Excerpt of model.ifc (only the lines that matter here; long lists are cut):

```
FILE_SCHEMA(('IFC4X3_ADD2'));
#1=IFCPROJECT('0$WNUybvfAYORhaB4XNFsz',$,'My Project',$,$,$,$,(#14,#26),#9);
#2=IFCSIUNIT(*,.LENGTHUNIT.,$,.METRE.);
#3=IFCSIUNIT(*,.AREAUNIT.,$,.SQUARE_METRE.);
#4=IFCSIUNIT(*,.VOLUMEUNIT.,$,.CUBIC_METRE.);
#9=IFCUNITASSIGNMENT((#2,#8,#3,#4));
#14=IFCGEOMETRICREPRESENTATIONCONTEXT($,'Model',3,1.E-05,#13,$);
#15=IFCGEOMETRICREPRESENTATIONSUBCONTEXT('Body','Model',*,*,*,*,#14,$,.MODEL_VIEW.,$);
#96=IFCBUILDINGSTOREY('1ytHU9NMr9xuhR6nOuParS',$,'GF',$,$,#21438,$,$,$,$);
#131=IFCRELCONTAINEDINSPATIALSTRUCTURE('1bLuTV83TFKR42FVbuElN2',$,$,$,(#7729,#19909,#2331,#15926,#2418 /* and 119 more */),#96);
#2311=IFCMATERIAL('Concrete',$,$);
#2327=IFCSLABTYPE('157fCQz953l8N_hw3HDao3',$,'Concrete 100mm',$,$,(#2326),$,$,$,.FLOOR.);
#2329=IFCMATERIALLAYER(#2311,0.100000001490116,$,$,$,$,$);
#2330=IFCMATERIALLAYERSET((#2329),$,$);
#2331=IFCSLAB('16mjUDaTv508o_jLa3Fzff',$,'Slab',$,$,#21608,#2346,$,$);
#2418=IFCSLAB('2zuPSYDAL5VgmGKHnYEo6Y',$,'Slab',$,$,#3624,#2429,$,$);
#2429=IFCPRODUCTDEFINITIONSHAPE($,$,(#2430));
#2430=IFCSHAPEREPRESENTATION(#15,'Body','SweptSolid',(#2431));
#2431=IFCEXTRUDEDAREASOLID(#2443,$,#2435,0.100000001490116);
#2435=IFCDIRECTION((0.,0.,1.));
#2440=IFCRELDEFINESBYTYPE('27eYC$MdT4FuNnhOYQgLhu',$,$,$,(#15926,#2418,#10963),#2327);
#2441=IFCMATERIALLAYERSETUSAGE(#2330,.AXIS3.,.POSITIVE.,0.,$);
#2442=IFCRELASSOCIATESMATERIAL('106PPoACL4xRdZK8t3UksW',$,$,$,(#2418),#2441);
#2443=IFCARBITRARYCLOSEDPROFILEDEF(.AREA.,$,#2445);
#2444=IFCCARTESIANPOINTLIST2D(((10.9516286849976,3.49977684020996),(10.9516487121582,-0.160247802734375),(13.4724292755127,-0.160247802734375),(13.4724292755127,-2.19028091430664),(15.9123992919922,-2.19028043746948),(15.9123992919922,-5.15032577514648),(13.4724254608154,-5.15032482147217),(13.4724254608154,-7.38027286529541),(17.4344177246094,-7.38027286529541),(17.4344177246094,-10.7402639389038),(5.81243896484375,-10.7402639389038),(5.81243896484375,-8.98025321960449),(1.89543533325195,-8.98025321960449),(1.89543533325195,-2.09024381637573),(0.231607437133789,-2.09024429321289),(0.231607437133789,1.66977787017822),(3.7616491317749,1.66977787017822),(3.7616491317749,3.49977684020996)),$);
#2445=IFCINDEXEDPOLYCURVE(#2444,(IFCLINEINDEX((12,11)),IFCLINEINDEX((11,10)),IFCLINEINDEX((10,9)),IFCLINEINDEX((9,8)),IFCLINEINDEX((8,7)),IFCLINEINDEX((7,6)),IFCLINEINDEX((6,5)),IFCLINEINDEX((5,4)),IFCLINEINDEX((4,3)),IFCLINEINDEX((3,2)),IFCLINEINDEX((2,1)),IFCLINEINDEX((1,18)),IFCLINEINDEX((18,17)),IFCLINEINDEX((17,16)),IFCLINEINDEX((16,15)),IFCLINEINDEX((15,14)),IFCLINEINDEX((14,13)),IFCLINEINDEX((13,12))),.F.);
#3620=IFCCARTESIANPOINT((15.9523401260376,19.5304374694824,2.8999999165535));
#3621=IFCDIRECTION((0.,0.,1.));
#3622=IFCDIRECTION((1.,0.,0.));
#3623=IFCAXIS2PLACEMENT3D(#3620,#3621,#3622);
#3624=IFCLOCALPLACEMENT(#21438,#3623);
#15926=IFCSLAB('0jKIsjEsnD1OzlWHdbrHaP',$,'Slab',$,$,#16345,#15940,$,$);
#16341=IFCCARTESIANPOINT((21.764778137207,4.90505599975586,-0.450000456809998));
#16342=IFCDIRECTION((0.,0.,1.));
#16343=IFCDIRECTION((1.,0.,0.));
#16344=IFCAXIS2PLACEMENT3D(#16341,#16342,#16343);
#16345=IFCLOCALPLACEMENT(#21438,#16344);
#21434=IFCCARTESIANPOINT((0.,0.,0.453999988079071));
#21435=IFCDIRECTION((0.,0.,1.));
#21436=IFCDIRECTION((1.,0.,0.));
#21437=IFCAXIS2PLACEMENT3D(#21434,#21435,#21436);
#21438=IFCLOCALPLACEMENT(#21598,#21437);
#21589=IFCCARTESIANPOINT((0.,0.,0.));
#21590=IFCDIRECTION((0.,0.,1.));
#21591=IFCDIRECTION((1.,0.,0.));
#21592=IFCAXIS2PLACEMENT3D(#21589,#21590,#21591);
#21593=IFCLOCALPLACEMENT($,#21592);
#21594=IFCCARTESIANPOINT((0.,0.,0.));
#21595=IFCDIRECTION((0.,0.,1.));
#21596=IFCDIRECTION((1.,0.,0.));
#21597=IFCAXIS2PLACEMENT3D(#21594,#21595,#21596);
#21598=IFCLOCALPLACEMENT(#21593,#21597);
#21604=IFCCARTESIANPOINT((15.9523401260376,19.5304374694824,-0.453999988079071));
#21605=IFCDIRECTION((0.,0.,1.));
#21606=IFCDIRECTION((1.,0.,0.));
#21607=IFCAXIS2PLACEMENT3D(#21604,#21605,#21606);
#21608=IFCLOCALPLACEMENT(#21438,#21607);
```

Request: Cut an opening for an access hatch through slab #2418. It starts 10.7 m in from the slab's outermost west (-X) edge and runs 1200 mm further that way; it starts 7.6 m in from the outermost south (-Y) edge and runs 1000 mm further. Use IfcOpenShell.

```python
import numpy as np
import ifcopenshell
import ifcopenshell.api.feature
import ifcopenshell.api.geometry
import ifcopenshell.api.root
import ifcopenshell.geom
import ifcopenshell.util.placement
import ifcopenshell.util.representation
import ifcopenshell.util.shape
import ifcopenshell.util.unit

model = ifcopenshell.open("model.ifc")
unit_scale = ifcopenshell.util.unit.calculate_unit_scale(model)
settings = ifcopenshell.geom.settings()


def volume(element):
    """Net volume in cubic metres, openings subtracted."""
    shape = ifcopenshell.geom.create_shape(settings, element)
    return ifcopenshell.util.shape.get_volume(shape.geometry)


slab = model.by_guid("2zuPSYDAL5VgmGKHnYEo6Y")
before = volume(slab)

# Extent in the slab's own axes, in metres. The edges named are its -X and -Y sides.
slab_shape = ifcopenshell.geom.create_shape(settings, slab)
vertices = ifcopenshell.util.shape.get_vertices(slab_shape.geometry)
x_min, y_min, bottom = vertices.min(axis=0)
top = vertices[:, 2].max()

opening = ifcopenshell.api.root.create_entity(model, ifc_class="IfcOpeningElement", name="Access hatch opening", predefined_type="OPENING")
context = ifcopenshell.util.representation.get_context(model, "Model", "Body", "MODEL_VIEW")
width, depth = 1.2, 1
outline = [(0.0, 0.0), (width, 0.0), (width, depth), (0.0, depth), (0.0, 0.0)]
# Overshoot both faces by 50 mm so the cut is clean.
shape = ifcopenshell.api.geometry.add_slab_representation(
    model, context=context, depth=top - bottom + 0.1, polyline=outline
)
ifcopenshell.api.geometry.assign_representation(model, product=opening, representation=shape)

matrix = ifcopenshell.util.placement.get_local_placement(slab.ObjectPlacement)
matrix[:, 3] = matrix @ np.append(np.array([x_min + 10.7, y_min + 7.6, bottom - 0.05]) / unit_scale, 1.0)
ifcopenshell.api.geometry.edit_object_placement(model, product=opening, matrix=matrix, is_si=False)
ifcopenshell.api.feature.add_feature(model, feature=opening, element=slab)

after = volume(slab)

print(f"slab volume {before:.3f} -> {after:.3f} m3")

model.write("model_edited.ifc")
```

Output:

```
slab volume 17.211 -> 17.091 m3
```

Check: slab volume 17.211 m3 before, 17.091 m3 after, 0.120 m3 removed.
